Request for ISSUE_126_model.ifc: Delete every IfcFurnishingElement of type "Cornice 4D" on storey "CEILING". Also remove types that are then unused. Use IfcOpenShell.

First a look at what the model holds.

```python
import ifcopenshell
import ifcopenshell.util.element

model = ifcopenshell.open("ISSUE_126_model.ifc")
print(model.schema)
storey = next(s for s in model.by_type("IfcBuildingStorey") if s.Name == "CEILING")
furniture = [e for e in ifcopenshell.util.element.get_decomposition(storey) if e.is_a("IfcFurnishingElement")]
seen = {}
for e in furniture:
    element_type = ifcopenshell.util.element.get_type(e)
    name = element_type.Name if element_type not in (None, e) else None
    seen[name] = seen.get(name, 0) + 1
for name, count in sorted(seen.items(), key=str):
    print(count, "x", name)
```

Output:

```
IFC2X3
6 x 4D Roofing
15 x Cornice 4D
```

```python
import ifcopenshell
import ifcopenshell.api.root
import ifcopenshell.util.element

model = ifcopenshell.open("ISSUE_126_model.ifc")

storey = next(s for s in model.by_type("IfcBuildingStorey") if s.Name == "CEILING")
furniture = [e for e in ifcopenshell.util.element.get_decomposition(storey) if e.is_a("IfcFurnishingElement")]
targets = [e for e in furniture if (t := ifcopenshell.util.element.get_type(e)) not in (None, e) and t.Name == "Cornice 4D"]
types = {ifcopenshell.util.element.get_type(e) for e in targets} - {None, *targets}

for e in targets:
    ifcopenshell.api.root.remove_product(model, product=e)
print(len(targets), "removed")

unused = [t for t in types if not ifcopenshell.util.element.get_types(t)]
for t in unused:
    ifcopenshell.api.root.remove_product(model, product=t)
print(len(unused), "unused types removed")

model.write("ISSUE_126_model_edited.ifc")
```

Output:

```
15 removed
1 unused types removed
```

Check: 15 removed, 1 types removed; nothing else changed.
